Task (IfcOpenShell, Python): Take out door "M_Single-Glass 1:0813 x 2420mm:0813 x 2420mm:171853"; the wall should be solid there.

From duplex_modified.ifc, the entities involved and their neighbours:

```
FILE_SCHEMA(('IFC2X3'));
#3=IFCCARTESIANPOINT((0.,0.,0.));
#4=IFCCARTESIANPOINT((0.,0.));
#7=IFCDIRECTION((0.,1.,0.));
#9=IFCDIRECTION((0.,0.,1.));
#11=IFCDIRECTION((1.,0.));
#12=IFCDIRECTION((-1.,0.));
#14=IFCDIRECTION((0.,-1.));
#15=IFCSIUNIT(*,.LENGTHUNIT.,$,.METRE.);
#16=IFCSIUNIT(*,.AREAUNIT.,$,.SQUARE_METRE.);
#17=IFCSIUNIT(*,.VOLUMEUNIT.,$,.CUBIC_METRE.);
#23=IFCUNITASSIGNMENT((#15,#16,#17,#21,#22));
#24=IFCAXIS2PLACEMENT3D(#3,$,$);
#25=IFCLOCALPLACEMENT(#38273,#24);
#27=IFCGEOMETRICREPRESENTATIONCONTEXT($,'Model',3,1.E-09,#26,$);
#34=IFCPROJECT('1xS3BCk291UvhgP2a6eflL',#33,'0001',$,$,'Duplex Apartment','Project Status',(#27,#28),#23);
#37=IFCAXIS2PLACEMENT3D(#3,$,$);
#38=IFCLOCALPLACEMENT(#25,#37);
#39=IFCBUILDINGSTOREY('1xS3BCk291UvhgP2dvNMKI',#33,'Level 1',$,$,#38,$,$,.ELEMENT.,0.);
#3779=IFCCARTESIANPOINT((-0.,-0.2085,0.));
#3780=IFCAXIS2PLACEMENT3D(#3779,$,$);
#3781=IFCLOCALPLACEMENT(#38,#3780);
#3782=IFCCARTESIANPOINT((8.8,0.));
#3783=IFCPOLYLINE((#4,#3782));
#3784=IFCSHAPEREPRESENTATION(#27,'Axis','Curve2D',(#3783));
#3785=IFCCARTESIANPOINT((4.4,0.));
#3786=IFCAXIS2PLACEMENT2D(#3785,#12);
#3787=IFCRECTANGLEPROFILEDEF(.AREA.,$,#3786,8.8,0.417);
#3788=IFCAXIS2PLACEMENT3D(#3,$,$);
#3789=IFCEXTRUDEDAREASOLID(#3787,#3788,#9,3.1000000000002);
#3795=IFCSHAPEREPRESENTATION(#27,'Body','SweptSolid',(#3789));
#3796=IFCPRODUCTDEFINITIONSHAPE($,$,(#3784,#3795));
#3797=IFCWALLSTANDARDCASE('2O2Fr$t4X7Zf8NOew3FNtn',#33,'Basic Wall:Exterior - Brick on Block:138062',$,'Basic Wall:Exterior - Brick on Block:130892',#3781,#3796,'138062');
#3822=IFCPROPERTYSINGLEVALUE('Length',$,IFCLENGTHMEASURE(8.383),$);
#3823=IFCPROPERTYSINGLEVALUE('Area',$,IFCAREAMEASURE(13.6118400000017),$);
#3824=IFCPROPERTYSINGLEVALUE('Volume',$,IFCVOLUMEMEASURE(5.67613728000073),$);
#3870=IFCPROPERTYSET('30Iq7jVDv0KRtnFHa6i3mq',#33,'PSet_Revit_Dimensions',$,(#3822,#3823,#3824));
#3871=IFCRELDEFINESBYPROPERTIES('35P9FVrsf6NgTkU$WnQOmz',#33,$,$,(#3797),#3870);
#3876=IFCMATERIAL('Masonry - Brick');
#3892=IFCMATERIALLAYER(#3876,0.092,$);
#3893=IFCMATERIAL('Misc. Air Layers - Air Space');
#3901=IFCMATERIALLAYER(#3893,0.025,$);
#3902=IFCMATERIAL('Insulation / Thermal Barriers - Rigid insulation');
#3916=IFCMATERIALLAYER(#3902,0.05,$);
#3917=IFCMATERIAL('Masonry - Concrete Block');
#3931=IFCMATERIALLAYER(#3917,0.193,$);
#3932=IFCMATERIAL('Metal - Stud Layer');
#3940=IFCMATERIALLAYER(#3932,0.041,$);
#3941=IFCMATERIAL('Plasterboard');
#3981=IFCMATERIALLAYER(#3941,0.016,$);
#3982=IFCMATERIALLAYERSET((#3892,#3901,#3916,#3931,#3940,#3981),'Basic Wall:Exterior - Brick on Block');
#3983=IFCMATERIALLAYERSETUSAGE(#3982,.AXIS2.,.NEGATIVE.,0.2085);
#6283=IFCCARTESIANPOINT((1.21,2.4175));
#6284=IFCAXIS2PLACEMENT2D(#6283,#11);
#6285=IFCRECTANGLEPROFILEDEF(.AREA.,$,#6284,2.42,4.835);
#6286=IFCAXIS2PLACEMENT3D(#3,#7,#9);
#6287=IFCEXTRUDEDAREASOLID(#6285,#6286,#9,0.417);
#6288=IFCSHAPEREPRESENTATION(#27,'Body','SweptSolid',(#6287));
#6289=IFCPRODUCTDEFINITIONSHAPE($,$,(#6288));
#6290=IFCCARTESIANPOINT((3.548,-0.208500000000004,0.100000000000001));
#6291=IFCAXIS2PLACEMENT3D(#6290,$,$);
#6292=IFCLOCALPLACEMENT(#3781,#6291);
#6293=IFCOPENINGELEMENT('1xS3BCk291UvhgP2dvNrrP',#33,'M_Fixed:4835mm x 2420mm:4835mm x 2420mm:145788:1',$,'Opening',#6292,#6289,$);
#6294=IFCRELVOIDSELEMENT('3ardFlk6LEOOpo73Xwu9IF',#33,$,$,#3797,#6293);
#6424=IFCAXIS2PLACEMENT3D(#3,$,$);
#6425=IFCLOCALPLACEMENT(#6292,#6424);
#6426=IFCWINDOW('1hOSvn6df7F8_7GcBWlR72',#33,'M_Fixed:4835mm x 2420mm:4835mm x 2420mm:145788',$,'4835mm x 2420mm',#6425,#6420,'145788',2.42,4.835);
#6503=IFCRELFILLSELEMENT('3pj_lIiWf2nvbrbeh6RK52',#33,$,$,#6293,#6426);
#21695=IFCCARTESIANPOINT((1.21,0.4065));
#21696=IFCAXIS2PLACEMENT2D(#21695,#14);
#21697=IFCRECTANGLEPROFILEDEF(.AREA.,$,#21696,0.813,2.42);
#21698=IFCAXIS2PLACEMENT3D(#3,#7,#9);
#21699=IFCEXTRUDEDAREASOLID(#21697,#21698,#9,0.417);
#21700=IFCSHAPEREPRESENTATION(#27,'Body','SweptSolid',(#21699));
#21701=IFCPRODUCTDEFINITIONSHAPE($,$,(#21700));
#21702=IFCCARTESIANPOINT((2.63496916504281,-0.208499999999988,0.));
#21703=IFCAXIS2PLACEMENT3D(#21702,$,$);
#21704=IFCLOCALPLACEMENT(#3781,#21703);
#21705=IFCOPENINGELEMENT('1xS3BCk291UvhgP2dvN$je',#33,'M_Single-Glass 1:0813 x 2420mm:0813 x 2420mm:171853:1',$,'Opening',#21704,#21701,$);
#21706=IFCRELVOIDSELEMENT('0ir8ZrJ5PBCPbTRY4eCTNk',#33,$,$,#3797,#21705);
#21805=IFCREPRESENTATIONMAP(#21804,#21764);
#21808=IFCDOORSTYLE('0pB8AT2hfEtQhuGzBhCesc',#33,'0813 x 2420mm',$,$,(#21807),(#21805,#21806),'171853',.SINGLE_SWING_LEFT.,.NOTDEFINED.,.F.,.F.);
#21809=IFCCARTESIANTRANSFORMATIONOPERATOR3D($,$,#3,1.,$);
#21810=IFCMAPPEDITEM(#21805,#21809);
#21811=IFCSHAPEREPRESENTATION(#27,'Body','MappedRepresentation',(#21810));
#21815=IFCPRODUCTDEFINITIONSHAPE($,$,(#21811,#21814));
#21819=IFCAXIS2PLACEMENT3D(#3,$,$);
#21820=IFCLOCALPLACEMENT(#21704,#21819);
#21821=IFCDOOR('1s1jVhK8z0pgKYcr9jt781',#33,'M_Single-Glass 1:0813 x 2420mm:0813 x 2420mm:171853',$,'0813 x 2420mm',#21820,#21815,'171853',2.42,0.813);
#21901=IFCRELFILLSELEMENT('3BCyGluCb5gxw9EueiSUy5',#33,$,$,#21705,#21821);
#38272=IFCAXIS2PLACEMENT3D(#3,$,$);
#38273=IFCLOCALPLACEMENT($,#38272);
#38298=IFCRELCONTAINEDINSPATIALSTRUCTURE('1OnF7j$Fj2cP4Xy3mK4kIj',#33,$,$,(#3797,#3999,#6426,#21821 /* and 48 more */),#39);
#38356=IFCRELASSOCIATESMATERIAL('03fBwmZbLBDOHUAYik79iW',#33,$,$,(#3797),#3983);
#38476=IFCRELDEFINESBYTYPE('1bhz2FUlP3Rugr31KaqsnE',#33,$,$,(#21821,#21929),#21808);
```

```python
import ifcopenshell
import ifcopenshell.api.feature
import ifcopenshell.api.pset
import ifcopenshell.api.root
import ifcopenshell.geom
import ifcopenshell.util.element
import ifcopenshell.util.shape
import ifcopenshell.util.unit

model = ifcopenshell.open("duplex_modified.ifc")
area_scale = ifcopenshell.util.unit.calculate_unit_scale(model, "AREAUNIT")
volume_scale = ifcopenshell.util.unit.calculate_unit_scale(model, "VOLUMEUNIT")
settings = ifcopenshell.geom.settings()


def volume(element):
    """Net volume in cubic metres, openings subtracted."""
    shape = ifcopenshell.geom.create_shape(settings, element)
    return ifcopenshell.util.shape.get_volume(shape.geometry)


door = model.by_guid("1s1jVhK8z0pgKYcr9jt781")
opening = door.FillsVoids[0].RelatingOpeningElement
wall = opening.VoidsElements[0].RelatingBuildingElement
before = volume(wall)

ifcopenshell.api.root.remove_product(model, product=door)
ifcopenshell.api.feature.remove_feature(model, feature=opening)

after = volume(wall)
thickness = 0.417  # wall thickness in metres

# Update the wall's stored quantities.
pset = model.by_id(ifcopenshell.util.element.get_pset(wall, "PSet_Revit_Dimensions", should_inherit=False)["id"])
ifcopenshell.api.pset.edit_pset(model, pset=pset, properties={
    "Area": model.create_entity("IfcAreaMeasure", after / thickness / area_scale),
    "Volume": model.create_entity("IfcVolumeMeasure", after / volume_scale),
})

print(f"wall volume {before:.3f} -> {after:.3f} m3")

model.write("duplex_modified-out.ifc")
```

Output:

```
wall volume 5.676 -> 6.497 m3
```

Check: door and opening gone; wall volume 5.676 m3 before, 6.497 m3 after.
